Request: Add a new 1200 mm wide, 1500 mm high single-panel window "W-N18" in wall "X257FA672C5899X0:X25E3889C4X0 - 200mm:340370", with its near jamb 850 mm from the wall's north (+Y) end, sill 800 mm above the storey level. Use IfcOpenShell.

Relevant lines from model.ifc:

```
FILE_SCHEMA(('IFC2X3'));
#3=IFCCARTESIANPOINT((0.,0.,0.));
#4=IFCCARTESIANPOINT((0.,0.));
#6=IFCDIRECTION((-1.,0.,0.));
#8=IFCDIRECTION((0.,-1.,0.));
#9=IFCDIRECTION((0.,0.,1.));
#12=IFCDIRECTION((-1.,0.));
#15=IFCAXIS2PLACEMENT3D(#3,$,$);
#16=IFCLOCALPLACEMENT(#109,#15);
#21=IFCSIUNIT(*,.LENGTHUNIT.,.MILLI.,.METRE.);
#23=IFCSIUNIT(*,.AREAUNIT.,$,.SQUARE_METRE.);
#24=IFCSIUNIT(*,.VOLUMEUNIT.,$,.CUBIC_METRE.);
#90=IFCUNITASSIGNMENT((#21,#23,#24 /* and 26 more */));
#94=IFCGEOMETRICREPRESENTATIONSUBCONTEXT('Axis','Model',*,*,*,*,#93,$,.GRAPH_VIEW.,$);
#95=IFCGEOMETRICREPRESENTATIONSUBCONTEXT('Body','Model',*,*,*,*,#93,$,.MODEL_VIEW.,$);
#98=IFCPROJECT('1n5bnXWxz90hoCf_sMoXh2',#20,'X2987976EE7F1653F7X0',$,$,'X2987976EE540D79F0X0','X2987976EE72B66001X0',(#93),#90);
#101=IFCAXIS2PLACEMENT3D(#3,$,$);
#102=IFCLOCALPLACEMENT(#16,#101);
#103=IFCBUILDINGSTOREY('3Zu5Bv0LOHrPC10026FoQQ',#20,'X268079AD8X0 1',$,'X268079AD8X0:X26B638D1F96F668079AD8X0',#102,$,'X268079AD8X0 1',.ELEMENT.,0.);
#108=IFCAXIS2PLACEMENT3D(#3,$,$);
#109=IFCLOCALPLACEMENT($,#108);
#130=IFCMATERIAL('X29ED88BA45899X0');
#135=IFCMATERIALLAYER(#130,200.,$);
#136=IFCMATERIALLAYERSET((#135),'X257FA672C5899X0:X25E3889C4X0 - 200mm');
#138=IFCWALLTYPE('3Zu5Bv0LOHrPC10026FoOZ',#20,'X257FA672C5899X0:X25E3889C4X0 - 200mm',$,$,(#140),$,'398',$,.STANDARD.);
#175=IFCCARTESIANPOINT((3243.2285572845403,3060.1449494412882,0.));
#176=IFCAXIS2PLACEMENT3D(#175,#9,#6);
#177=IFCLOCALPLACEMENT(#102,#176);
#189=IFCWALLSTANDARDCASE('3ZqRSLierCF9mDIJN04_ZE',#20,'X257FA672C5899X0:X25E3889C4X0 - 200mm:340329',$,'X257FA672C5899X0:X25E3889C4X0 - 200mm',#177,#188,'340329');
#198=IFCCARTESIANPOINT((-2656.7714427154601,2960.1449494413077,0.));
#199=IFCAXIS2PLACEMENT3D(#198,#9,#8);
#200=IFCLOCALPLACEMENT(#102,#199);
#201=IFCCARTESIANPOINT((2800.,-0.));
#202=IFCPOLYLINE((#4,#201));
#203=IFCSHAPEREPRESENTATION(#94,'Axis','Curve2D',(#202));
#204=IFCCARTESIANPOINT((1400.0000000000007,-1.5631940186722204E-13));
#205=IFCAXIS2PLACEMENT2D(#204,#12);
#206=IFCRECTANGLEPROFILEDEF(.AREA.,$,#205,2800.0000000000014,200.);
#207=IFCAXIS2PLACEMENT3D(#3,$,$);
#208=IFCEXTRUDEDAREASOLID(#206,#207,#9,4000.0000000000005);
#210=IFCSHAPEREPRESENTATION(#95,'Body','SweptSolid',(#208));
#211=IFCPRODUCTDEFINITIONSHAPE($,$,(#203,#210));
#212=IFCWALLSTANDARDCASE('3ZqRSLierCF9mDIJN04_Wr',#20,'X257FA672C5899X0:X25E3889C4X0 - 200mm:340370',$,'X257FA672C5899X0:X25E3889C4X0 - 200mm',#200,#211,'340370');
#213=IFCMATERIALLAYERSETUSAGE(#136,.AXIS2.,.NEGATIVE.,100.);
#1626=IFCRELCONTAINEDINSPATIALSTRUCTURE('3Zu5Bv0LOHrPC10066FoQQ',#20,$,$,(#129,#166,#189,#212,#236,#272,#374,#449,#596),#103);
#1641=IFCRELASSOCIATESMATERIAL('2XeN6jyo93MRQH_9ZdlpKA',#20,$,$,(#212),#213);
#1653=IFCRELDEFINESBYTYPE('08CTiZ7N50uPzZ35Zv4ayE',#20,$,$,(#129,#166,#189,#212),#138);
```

```python
import numpy as np
import ifcopenshell
import ifcopenshell.api.feature
import ifcopenshell.api.geometry
import ifcopenshell.api.root
import ifcopenshell.api.spatial
import ifcopenshell.api.type
import ifcopenshell.geom
import ifcopenshell.util.element
import ifcopenshell.util.placement
import ifcopenshell.util.representation
import ifcopenshell.util.shape
import ifcopenshell.util.unit

model = ifcopenshell.open("model.ifc")
unit_scale = ifcopenshell.util.unit.calculate_unit_scale(model)
settings = ifcopenshell.geom.settings()


def volume(element):
    """Net volume in cubic metres, openings subtracted."""
    shape = ifcopenshell.geom.create_shape(settings, element)
    return ifcopenshell.util.shape.get_volume(shape.geometry)


wall = model.by_guid("3ZqRSLierCF9mDIJN04_Wr")
storey = ifcopenshell.util.element.get_container(wall, ifc_class="IfcBuildingStorey")
context = ifcopenshell.util.representation.get_context(model, "Model", "Body", "MODEL_VIEW")
before = volume(wall)

width, height, from_end, sill = 1.2, 1.5, 0.85, 0.8  # metres

# The wall runs along its own X axis, and the end named is its -X end.
wall_shape = ifcopenshell.geom.create_shape(settings, wall)
x, y, z = ifcopenshell.util.shape.get_vertices(wall_shape.geometry).T
start = x.min() + from_end
face, thickness = float(y.min()), float(y.max() - y.min())
wall_matrix = ifcopenshell.util.placement.get_local_placement(wall.ObjectPlacement)
level = ifcopenshell.util.placement.get_local_placement(storey.ObjectPlacement)[2, 3]


def in_wall(x, y):
    """Placement at x, y metres in the wall's axes, at sill height."""
    matrix = wall_matrix.copy()
    matrix[:, 3] = wall_matrix @ np.array([x / unit_scale, y / unit_scale, 0.0, 1.0])
    matrix[2, 3] = level + sill / unit_scale
    return matrix


# Opening: a box that overshoots both wall faces by 50 mm.
opening = ifcopenshell.api.root.create_entity(model, ifc_class="IfcOpeningElement")
box = ifcopenshell.api.geometry.add_wall_representation(
    model, context=context, length=width, height=height, thickness=thickness + 0.1
)
ifcopenshell.api.geometry.assign_representation(model, product=opening, representation=box)
ifcopenshell.api.geometry.edit_object_placement(model, product=opening, matrix=in_wall(start, face - 0.05), is_si=False)
ifcopenshell.api.feature.add_feature(model, feature=opening, element=wall)

window = ifcopenshell.api.root.create_entity(model, ifc_class="IfcWindow", name="W-N18")
window.OverallWidth, window.OverallHeight = width / unit_scale, height / unit_scale
body = ifcopenshell.api.geometry.add_window_representation(
    model,
    context=context,
    overall_width=window.OverallWidth,
    overall_height=window.OverallHeight,
    partition_type="SINGLE_PANEL",
)
ifcopenshell.api.geometry.assign_representation(model, product=window, representation=body)
ifcopenshell.api.spatial.assign_container(model, products=[window], relating_structure=storey)
fills = ifcopenshell.api.feature.add_filling(model, opening=opening, element=window)
fills.OwnerHistory = window.OwnerHistory  # required in IFC2X3

# IFC2X3 keeps the operation on the window style.
style = ifcopenshell.api.root.create_entity(model, ifc_class="IfcWindowStyle", name="W-N18")
style.OperationType, style.ConstructionType = "SINGLE_PANEL", "NOTDEFINED"
style.ParameterTakesPrecedence = style.Sizeable = False
ifcopenshell.api.type.assign_type(model, related_objects=[window], relating_type=style)

# Centre the window in the wall's thickness.
ifcopenshell.api.geometry.edit_object_placement(model, product=window, matrix=in_wall(start, face), is_si=False)
window_shape = ifcopenshell.geom.create_shape(settings, window)
depth = ifcopenshell.util.shape.get_vertices(window_shape.geometry)[:, 1]
offset = face + thickness / 2 - (depth.min() + depth.max()) / 2
ifcopenshell.api.geometry.edit_object_placement(model, product=window, matrix=in_wall(start, offset), is_si=False)

after = volume(wall)

print(f"wall volume {before:.3f} -> {after:.3f} m3")

model.write("model_v2.ifc")
```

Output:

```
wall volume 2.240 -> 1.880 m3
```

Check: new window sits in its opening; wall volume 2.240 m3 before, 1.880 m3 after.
